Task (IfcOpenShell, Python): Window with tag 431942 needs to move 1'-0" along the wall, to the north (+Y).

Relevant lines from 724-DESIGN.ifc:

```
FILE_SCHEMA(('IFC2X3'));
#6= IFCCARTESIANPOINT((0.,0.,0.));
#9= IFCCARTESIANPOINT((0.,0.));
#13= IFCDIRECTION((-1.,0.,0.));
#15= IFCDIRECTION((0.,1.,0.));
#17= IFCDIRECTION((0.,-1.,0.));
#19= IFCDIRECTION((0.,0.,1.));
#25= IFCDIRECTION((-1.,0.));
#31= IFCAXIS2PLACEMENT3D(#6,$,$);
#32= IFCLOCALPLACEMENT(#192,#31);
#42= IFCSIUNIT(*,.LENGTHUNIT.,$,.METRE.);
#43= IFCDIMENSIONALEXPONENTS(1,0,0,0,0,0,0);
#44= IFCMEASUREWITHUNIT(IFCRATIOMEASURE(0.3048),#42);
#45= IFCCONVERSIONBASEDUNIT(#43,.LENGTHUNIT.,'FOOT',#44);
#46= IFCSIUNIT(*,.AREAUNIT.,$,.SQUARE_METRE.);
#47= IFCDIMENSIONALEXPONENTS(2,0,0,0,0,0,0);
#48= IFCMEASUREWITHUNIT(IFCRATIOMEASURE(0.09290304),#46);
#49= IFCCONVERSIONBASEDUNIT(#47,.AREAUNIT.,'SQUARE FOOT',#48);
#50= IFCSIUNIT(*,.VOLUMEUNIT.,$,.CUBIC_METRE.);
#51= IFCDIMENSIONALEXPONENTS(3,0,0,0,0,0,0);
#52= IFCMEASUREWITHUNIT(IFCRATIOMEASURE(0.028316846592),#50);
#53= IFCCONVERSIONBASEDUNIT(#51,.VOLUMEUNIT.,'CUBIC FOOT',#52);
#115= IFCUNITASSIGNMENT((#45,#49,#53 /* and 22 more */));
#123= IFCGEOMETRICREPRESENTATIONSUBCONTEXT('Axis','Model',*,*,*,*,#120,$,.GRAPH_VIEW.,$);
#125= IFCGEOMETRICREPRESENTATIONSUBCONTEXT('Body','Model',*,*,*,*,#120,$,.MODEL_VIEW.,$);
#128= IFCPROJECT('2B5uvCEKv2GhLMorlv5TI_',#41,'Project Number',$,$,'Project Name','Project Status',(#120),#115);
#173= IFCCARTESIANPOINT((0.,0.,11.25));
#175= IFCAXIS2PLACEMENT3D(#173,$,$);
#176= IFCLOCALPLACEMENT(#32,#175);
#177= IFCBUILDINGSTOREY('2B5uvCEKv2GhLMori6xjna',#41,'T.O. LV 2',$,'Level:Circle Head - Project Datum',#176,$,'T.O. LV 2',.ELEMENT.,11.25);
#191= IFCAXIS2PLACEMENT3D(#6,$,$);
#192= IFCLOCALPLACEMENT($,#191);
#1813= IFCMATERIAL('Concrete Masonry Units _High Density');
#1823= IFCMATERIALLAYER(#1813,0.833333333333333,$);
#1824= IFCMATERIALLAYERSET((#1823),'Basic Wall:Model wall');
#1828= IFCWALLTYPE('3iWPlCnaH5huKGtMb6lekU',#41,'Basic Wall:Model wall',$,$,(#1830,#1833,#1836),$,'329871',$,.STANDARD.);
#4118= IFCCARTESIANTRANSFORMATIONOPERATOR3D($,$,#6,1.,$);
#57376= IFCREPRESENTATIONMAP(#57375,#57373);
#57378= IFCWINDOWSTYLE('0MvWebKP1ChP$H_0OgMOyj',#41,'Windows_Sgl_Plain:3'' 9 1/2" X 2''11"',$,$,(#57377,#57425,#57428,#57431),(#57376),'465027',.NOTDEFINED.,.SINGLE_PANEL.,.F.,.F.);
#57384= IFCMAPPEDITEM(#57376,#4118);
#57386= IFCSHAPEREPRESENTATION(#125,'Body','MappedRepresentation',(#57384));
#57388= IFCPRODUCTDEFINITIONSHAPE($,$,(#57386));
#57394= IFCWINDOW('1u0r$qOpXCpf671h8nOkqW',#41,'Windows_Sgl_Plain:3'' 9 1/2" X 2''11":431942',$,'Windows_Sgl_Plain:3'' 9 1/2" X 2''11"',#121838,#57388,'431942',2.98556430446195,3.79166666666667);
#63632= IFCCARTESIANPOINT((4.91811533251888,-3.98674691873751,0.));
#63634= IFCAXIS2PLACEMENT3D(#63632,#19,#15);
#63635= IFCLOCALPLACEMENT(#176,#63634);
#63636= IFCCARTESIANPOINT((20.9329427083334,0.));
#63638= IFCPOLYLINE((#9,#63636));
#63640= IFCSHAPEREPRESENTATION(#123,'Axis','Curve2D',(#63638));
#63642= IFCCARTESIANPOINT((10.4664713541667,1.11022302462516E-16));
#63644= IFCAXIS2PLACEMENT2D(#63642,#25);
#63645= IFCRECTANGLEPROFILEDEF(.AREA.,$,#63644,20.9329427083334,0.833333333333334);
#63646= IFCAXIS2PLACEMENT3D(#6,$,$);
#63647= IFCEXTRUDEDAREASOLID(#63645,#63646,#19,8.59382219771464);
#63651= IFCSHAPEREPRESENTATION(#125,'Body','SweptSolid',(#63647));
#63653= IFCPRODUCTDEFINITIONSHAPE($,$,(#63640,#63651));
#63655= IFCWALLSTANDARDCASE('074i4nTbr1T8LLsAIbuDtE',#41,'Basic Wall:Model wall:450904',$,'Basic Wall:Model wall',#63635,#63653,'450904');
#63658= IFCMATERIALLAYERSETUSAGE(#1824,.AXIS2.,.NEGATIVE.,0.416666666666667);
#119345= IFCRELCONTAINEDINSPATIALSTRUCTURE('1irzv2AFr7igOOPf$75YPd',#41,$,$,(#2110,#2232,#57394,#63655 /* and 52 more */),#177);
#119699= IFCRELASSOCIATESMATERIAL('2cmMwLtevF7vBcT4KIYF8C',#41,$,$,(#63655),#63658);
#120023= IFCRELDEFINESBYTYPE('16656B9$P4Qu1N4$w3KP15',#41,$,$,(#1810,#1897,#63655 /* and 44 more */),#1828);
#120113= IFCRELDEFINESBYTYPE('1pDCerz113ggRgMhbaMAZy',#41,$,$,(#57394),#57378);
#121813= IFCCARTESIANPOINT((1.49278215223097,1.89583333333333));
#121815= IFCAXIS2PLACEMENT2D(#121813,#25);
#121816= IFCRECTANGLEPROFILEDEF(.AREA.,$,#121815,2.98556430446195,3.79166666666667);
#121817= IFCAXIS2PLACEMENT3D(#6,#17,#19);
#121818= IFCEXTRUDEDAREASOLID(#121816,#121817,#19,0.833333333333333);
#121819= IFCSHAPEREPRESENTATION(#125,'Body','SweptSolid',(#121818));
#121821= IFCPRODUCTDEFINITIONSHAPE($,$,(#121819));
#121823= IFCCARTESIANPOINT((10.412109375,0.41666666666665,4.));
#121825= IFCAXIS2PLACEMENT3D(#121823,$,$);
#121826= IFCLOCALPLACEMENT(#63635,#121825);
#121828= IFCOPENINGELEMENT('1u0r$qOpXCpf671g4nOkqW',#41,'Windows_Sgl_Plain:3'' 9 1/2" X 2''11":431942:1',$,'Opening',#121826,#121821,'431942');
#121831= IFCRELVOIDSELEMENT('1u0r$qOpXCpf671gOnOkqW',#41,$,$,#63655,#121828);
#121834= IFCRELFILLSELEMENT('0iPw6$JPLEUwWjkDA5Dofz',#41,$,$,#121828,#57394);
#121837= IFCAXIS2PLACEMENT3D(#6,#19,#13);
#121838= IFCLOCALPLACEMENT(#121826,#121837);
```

```python
import ifcopenshell
import ifcopenshell.api.geometry
import ifcopenshell.util.placement
import ifcopenshell.util.unit

model = ifcopenshell.open("724-DESIGN.ifc")
unit_scale = ifcopenshell.util.unit.calculate_unit_scale(model)

window = model.by_guid("1u0r$qOpXCpf671h8nOkqW")
opening = window.FillsVoids[0].RelatingOpeningElement
wall = opening.VoidsElements[0].RelatingBuildingElement

wall_matrix = ifcopenshell.util.placement.get_local_placement(wall.ObjectPlacement)
shift = wall_matrix[:3, 0] * 12 * 0.0254 / unit_scale
before = ifcopenshell.util.placement.get_local_placement(window.ObjectPlacement)[:3, 3].copy()

# The window is placed relative to its opening, so it follows when the opening moves.
matrix = ifcopenshell.util.placement.get_local_placement(opening.ObjectPlacement)
matrix[:3, 3] += shift
ifcopenshell.api.geometry.edit_object_placement(
    model, product=opening, matrix=matrix, is_si=False, should_transform_children=True
)

after = ifcopenshell.util.placement.get_local_placement(window.ObjectPlacement)[:3, 3]
print("window moved by", (after - before).round(3) + 0.0)

model.write("724-DESIGN_v2.ifc")
```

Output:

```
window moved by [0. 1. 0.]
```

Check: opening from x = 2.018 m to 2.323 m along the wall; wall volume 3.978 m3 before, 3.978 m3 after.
